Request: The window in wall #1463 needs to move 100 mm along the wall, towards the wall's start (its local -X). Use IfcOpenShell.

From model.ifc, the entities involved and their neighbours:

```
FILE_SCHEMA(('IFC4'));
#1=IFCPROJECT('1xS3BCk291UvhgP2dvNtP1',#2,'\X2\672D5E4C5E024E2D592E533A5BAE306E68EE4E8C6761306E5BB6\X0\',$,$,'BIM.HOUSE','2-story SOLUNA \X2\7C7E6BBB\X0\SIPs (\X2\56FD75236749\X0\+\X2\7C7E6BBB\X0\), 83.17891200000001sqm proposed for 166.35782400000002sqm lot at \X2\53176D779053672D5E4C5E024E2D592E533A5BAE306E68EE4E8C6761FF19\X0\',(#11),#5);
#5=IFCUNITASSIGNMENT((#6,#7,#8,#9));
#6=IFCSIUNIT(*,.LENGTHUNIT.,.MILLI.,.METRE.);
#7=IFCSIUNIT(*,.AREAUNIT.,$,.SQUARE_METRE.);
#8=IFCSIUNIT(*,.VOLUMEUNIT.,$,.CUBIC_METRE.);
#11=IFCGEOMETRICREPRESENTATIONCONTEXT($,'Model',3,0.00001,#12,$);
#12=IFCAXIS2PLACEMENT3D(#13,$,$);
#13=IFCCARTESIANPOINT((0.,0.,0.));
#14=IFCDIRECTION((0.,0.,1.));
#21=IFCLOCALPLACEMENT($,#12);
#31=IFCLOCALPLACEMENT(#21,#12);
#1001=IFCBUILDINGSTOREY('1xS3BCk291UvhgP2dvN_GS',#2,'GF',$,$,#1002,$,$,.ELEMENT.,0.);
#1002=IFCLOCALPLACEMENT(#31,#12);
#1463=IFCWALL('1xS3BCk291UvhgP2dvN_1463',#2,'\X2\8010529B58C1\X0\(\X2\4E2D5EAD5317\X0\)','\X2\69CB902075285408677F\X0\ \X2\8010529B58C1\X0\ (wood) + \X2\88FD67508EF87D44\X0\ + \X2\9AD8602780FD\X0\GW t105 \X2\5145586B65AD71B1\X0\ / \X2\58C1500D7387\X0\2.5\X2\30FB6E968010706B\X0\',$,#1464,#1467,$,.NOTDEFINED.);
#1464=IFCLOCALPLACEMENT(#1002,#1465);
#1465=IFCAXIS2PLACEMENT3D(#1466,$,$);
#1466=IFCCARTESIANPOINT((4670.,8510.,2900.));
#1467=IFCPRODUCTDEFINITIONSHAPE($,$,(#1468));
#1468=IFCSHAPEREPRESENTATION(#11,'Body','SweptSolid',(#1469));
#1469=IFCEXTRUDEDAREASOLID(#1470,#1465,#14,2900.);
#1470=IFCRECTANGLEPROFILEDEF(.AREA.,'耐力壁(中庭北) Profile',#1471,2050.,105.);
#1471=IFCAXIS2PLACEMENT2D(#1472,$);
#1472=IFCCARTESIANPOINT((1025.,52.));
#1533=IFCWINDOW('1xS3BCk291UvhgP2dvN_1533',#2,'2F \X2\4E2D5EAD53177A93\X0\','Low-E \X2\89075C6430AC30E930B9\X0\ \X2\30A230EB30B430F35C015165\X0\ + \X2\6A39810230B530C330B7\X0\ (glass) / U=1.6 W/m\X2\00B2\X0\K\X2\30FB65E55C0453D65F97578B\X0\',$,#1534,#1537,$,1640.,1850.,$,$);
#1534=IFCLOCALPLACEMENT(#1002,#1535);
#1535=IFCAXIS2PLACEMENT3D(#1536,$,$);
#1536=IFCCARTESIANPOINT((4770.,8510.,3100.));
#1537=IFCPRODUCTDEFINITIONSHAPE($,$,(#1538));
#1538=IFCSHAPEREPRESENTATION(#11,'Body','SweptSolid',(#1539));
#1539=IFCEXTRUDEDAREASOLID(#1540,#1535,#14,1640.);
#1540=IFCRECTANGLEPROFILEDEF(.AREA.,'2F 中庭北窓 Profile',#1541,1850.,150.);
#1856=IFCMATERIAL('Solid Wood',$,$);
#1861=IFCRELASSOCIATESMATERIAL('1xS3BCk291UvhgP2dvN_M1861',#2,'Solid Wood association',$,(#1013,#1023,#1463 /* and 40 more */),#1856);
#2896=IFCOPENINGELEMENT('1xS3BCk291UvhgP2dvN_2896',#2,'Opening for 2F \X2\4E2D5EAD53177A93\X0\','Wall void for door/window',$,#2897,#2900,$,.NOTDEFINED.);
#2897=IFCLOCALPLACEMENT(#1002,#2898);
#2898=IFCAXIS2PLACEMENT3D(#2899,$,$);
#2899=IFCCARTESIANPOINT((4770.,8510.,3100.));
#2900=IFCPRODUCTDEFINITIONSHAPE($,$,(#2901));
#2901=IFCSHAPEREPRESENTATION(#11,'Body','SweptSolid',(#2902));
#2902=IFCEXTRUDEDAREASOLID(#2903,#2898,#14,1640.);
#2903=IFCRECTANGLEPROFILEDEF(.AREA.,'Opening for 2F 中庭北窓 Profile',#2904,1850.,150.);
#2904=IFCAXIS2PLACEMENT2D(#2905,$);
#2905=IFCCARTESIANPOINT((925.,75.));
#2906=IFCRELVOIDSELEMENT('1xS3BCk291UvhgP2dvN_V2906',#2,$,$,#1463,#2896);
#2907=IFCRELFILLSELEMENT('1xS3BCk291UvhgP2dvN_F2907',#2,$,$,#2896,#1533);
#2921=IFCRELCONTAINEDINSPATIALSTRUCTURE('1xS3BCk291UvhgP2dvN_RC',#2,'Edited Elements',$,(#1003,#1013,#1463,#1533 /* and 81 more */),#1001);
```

```python
import ifcopenshell
import ifcopenshell.api.geometry
import ifcopenshell.util.placement
import ifcopenshell.util.unit

model = ifcopenshell.open("model.ifc")
unit_scale = ifcopenshell.util.unit.calculate_unit_scale(model)

window = model.by_guid("1xS3BCk291UvhgP2dvN_1533")
opening = window.FillsVoids[0].RelatingOpeningElement
wall = opening.VoidsElements[0].RelatingBuildingElement

wall_matrix = ifcopenshell.util.placement.get_local_placement(wall.ObjectPlacement)
shift = wall_matrix[:3, 0] * -0.1 / unit_scale
before = ifcopenshell.util.placement.get_local_placement(window.ObjectPlacement)[:3, 3].copy()

# The window is not placed relative to its opening, so move both.
for product in (opening, window):
    matrix = ifcopenshell.util.placement.get_local_placement(product.ObjectPlacement)
    matrix[:3, 3] += shift
    ifcopenshell.api.geometry.edit_object_placement(model, product=product, matrix=matrix, is_si=False)

after = ifcopenshell.util.placement.get_local_placement(window.ObjectPlacement)[:3, 3]
print("window moved by", (after - before).round(3) + 0.0)

model.write("model_v2.ifc")
```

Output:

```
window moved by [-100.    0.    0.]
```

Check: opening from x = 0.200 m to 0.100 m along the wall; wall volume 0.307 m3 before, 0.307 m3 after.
